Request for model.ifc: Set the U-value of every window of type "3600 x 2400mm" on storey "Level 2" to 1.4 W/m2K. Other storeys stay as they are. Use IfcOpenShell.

First a look at what the model holds.

```python
import ifcopenshell
import ifcopenshell.util.element

model = ifcopenshell.open("model.ifc")
print(model.schema)
storey = next(s for s in model.by_type("IfcBuildingStorey") if s.Name == "Level 2")
windows = [e for e in ifcopenshell.util.element.get_decomposition(storey) if e.is_a("IfcWindow")]
seen = {}
for e in windows:
    element_type = ifcopenshell.util.element.get_type(e)
    key = (element_type.Name if element_type != e and element_type else None, ifcopenshell.util.element.get_pset(e, "Pset_WindowCommon", "ThermalTransmittance"))
    seen[key] = seen.get(key, 0) + 1
for (name, value), count in sorted(seen.items(), key=str):
    print(count, "x", name, "|", value)
```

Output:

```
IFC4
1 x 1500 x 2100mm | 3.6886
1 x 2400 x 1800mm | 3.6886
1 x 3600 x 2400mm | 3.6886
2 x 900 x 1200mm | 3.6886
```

```python
import ifcopenshell
import ifcopenshell.api.pset
import ifcopenshell.util.element

model = ifcopenshell.open("model.ifc")

storey = next(s for s in model.by_type("IfcBuildingStorey") if s.Name == "Level 2")
windows = [e for e in ifcopenshell.util.element.get_decomposition(storey) if e.is_a("IfcWindow")]

count = 0
for e in windows:
    element_type = ifcopenshell.util.element.get_type(e)
    if element_type in (None, e) or element_type.Name != "3600 x 2400mm":
        continue
    # add_pset returns the element's existing set when there is one.
    pset = ifcopenshell.api.pset.add_pset(model, product=e, name="Pset_WindowCommon")
    ifcopenshell.api.pset.edit_pset(model, pset=pset, properties={"ThermalTransmittance": 1.4})
    count += 1

print(count, "windows updated")

model.write("model_v2.ifc")
```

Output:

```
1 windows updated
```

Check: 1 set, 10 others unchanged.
